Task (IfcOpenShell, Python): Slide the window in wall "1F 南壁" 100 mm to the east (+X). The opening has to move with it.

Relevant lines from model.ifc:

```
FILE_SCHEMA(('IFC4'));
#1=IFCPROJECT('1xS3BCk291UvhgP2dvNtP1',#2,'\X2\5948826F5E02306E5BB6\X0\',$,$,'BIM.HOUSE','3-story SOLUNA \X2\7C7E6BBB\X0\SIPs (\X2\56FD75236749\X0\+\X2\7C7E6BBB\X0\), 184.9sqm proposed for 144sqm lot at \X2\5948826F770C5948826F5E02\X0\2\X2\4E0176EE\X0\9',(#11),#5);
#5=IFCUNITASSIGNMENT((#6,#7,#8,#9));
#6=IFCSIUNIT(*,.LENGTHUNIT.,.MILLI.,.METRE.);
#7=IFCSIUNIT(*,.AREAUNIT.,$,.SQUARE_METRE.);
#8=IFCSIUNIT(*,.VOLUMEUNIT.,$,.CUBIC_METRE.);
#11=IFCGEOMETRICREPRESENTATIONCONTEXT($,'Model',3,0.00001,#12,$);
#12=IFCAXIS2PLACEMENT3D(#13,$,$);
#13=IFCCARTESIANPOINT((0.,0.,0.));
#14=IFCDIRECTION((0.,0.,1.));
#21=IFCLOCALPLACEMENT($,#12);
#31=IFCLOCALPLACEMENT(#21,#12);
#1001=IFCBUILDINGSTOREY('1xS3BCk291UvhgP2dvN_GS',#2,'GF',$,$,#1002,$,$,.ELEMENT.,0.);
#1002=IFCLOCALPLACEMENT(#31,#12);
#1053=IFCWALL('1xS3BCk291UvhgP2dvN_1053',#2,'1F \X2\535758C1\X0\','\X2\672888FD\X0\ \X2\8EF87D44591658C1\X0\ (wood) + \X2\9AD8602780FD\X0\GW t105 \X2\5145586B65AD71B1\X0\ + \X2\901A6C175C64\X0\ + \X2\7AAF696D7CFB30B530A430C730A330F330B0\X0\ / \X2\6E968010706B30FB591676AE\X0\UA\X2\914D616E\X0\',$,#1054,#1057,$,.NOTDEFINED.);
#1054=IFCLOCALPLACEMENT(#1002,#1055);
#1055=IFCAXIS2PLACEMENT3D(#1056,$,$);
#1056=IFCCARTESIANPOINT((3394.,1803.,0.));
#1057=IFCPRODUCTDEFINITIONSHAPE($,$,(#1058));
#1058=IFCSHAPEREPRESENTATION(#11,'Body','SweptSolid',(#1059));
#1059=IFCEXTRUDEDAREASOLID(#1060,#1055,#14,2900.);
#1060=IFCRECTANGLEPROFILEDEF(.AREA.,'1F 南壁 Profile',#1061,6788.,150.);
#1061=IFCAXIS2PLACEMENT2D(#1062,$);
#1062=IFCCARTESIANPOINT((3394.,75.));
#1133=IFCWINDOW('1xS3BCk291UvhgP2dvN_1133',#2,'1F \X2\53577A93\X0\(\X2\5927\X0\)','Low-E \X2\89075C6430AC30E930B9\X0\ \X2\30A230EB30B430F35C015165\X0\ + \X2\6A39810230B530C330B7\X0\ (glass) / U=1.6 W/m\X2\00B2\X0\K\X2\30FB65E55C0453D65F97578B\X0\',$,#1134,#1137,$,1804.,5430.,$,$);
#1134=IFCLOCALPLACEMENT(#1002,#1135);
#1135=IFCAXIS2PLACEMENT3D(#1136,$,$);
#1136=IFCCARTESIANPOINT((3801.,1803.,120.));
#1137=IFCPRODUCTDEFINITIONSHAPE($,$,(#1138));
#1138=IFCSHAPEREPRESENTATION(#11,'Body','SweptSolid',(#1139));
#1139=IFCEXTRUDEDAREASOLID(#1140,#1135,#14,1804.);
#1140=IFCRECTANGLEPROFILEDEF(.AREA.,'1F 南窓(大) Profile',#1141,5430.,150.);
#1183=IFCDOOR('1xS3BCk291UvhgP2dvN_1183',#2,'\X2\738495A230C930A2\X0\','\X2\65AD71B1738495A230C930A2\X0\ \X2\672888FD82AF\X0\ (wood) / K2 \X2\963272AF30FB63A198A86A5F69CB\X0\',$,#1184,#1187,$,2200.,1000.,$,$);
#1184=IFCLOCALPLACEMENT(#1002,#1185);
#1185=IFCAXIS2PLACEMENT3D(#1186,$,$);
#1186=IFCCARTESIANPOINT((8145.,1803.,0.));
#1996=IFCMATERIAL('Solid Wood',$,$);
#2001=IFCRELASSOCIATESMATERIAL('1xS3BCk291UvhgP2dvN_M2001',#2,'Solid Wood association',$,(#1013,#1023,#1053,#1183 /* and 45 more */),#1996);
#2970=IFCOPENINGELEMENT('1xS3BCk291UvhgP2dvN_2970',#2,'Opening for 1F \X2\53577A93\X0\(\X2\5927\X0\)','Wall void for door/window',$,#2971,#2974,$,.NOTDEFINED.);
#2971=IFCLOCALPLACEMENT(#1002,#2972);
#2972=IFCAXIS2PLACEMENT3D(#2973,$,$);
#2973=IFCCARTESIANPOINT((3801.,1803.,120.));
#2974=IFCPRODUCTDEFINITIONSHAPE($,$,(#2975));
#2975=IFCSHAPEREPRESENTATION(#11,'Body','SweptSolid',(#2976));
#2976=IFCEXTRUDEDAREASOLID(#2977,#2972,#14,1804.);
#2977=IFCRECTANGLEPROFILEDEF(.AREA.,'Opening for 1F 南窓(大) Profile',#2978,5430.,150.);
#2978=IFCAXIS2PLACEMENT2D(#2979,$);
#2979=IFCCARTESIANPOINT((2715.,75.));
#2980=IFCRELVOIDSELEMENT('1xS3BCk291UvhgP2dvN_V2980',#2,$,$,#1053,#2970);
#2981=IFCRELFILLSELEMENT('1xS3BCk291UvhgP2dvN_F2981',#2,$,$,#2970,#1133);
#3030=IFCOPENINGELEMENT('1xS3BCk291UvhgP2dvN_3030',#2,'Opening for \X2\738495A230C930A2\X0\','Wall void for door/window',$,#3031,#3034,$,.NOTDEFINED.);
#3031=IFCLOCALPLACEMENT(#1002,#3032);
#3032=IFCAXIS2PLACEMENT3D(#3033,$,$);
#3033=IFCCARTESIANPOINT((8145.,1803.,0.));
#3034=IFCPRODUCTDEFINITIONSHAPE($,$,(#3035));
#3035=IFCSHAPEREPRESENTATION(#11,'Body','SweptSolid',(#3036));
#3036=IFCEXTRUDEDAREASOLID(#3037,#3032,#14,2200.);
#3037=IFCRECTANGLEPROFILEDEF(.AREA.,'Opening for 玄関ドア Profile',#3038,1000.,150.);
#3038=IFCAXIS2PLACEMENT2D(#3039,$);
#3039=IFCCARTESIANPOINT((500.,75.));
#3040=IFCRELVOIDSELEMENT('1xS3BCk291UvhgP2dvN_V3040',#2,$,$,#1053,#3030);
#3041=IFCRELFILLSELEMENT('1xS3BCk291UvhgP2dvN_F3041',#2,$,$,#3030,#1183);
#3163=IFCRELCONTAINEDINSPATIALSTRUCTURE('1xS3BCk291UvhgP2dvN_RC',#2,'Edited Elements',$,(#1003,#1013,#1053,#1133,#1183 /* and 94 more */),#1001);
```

```python
import ifcopenshell
import ifcopenshell.api.geometry
import ifcopenshell.util.placement
import ifcopenshell.util.unit

model = ifcopenshell.open("model.ifc")
unit_scale = ifcopenshell.util.unit.calculate_unit_scale(model)

window = model.by_id(1133)
opening = window.FillsVoids[0].RelatingOpeningElement
wall = opening.VoidsElements[0].RelatingBuildingElement

wall_matrix = ifcopenshell.util.placement.get_local_placement(wall.ObjectPlacement)
shift = wall_matrix[:3, 0] * 0.1 / unit_scale
before = ifcopenshell.util.placement.get_local_placement(window.ObjectPlacement)[:3, 3].copy()

# The window is not placed relative to its opening, so move both.
for product in (opening, window):
    matrix = ifcopenshell.util.placement.get_local_placement(product.ObjectPlacement)
    matrix[:3, 3] += shift
    ifcopenshell.api.geometry.edit_object_placement(model, product=product, matrix=matrix, is_si=False)

after = ifcopenshell.util.placement.get_local_placement(window.ObjectPlacement)[:3, 3]
print("window moved by", (after - before).round(3) + 0.0)

model.write("model-out.ifc")
```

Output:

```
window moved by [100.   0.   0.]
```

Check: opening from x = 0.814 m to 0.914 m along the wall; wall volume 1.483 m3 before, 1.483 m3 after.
